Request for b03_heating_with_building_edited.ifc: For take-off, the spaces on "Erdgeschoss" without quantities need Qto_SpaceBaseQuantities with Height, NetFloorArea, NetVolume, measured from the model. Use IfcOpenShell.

First a look at what the model holds.

```python
import ifcopenshell
import ifcopenshell.util.element
import ifcopenshell.util.unit

model = ifcopenshell.open("b03_heating_with_building_edited.ifc")
print(model.schema)
for unit_type in ("LENGTHUNIT", "AREAUNIT", "VOLUMEUNIT"):
    print(unit_type, ifcopenshell.util.unit.calculate_unit_scale(model, unit_type))
storey = next(s for s in model.by_type("IfcBuildingStorey") if s.Name == "Erdgeschoss")
spaces = [e for e in ifcopenshell.util.element.get_decomposition(storey) if e.is_a("IfcSpace")]
for e in sorted(spaces, key=lambda e: e.id()):
    print(e.id(), e.is_a(), e.Name, list(ifcopenshell.util.element.get_psets(e, qtos_only=True)), sep=" | ")
```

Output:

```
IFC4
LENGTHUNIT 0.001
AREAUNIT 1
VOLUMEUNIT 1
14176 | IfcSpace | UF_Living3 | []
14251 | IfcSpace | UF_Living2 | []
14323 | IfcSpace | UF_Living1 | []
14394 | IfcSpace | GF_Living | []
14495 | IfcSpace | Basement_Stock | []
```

```python
import ifcopenshell
import ifcopenshell.api.pset
import ifcopenshell.geom
import ifcopenshell.util.element
import ifcopenshell.util.shape
import ifcopenshell.util.unit

model = ifcopenshell.open("b03_heating_with_building_edited.ifc")
unit_scale = ifcopenshell.util.unit.calculate_unit_scale(model)
area_scale = ifcopenshell.util.unit.calculate_unit_scale(model, "AREAUNIT")
volume_scale = ifcopenshell.util.unit.calculate_unit_scale(model, "VOLUMEUNIT")
settings = ifcopenshell.geom.settings()

storey = next(s for s in model.by_type("IfcBuildingStorey") if s.Name == "Erdgeschoss")
spaces = [e for e in ifcopenshell.util.element.get_decomposition(storey) if e.is_a("IfcSpace")]

for e in sorted(spaces, key=lambda e: e.id()):
    if ifcopenshell.util.element.get_psets(e, qtos_only=True, should_inherit=False):
        continue
    # Geometry comes back in metres, in the element's own axes.
    shape = ifcopenshell.geom.create_shape(settings, e)
    values = {
        "Height": ifcopenshell.util.shape.get_z(shape.geometry) / unit_scale,
        "NetFloorArea": ifcopenshell.util.shape.get_footprint_area(shape.geometry) / area_scale,
        "NetVolume": ifcopenshell.util.shape.get_volume(shape.geometry) / volume_scale,
    }
    qto = ifcopenshell.api.pset.add_qto(model, product=e, name="Qto_SpaceBaseQuantities")
    ifcopenshell.api.pset.edit_qto(model, qto=qto, properties=values)
    print(e.id(), {k: round(v, 3) for k, v in values.items()})

model.write("b03_heating_with_building_edited_edited.ifc")
```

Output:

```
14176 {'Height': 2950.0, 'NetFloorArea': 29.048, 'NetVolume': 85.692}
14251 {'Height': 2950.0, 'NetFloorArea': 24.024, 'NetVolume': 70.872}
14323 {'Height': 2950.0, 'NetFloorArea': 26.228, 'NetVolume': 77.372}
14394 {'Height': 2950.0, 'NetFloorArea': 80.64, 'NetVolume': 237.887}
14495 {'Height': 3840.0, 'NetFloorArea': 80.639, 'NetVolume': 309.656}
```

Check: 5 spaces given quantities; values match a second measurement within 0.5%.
